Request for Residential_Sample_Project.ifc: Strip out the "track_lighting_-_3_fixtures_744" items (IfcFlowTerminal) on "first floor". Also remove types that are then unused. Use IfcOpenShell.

First a look at what the model holds.

```python
import ifcopenshell
import ifcopenshell.util.element

model = ifcopenshell.open("Residential_Sample_Project.ifc")
print(model.schema)
storey = next(s for s in model.by_type("IfcBuildingStorey") if s.Name == "first floor")
terminals = [e for e in ifcopenshell.util.element.get_decomposition(storey) if e.is_a("IfcFlowTerminal")]
seen = {}
for e in terminals:
    element_type = ifcopenshell.util.element.get_type(e)
    name = element_type.Name if element_type not in (None, e) else None
    seen[name] = seen.get(name, 0) + 1
for name, count in sorted(seen.items(), key=str):
    print(count, "x", name)
```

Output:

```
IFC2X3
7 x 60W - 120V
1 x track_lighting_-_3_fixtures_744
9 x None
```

```python
import ifcopenshell
import ifcopenshell.api.root
import ifcopenshell.util.element

model = ifcopenshell.open("Residential_Sample_Project.ifc")

storey = next(s for s in model.by_type("IfcBuildingStorey") if s.Name == "first floor")
terminals = [e for e in ifcopenshell.util.element.get_decomposition(storey) if e.is_a("IfcFlowTerminal")]
targets = [e for e in terminals if (t := ifcopenshell.util.element.get_type(e)) not in (None, e) and t.Name == "track_lighting_-_3_fixtures_744"]
types = {ifcopenshell.util.element.get_type(e) for e in targets} - {None, *targets}

for e in targets:
    ifcopenshell.api.root.remove_product(model, product=e)
print(len(targets), "removed")

unused = [t for t in types if not ifcopenshell.util.element.get_types(t)]
for t in unused:
    ifcopenshell.api.root.remove_product(model, product=t)
print(len(unused), "unused types removed")

model.write("Residential_Sample_Project-out.ifc")
```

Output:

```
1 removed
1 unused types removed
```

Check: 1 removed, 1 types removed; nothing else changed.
